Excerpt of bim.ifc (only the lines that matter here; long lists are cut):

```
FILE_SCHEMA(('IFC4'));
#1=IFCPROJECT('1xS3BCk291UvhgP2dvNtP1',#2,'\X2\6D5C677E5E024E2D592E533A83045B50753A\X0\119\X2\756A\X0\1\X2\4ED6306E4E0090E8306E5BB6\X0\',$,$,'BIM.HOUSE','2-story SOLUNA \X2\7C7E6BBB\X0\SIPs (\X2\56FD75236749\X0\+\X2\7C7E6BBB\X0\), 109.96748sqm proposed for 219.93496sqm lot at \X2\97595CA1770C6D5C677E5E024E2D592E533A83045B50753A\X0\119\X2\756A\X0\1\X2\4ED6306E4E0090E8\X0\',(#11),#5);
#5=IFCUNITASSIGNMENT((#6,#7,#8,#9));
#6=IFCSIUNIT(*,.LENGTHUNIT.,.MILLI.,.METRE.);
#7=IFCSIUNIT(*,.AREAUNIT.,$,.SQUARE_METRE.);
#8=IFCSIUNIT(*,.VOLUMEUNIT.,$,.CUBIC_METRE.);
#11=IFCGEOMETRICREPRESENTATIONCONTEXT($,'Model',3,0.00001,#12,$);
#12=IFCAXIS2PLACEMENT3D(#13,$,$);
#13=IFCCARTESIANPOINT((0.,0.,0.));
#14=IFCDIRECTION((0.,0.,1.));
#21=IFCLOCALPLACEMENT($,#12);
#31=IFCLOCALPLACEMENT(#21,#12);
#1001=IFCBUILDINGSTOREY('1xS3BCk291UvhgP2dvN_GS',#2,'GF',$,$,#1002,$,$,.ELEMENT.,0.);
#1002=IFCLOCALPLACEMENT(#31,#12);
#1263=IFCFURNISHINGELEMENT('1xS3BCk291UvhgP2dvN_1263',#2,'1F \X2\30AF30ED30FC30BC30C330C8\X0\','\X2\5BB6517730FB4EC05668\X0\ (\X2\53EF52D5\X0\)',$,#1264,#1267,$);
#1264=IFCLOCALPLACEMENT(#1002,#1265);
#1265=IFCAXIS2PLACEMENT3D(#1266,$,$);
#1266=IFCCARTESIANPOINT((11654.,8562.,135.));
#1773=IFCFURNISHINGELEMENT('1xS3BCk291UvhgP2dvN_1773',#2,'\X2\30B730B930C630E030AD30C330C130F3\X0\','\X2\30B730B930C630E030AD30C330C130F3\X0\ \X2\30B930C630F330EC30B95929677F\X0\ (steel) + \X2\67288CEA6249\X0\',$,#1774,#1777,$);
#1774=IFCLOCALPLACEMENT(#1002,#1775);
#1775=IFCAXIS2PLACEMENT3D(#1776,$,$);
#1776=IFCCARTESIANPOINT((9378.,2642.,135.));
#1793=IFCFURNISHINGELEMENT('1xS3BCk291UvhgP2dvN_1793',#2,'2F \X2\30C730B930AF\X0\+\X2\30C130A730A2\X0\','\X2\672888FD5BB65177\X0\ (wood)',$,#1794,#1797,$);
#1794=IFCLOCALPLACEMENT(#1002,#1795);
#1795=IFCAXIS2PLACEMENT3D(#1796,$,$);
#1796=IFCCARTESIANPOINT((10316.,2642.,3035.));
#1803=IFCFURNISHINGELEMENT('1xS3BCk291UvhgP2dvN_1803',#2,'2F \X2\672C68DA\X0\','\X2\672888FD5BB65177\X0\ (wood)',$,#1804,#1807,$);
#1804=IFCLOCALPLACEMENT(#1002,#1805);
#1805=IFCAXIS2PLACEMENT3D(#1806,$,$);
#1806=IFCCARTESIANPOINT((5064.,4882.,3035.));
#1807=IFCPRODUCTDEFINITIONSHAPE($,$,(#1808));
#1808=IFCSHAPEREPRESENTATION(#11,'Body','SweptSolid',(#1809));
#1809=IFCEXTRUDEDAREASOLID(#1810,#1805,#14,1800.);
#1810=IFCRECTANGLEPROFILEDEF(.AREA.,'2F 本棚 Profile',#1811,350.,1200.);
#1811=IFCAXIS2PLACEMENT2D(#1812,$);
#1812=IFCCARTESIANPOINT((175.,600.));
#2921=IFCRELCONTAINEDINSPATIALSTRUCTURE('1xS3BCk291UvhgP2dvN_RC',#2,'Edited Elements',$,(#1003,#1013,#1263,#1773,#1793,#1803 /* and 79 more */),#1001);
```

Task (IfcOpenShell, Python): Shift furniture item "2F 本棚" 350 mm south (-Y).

```python
import ifcopenshell
import ifcopenshell.api.geometry
import ifcopenshell.util.placement
import ifcopenshell.util.unit

model = ifcopenshell.open("bim.ifc")
unit_scale = ifcopenshell.util.unit.calculate_unit_scale(model)

item = model.by_id(1803)
matrix = ifcopenshell.util.placement.get_local_placement(item.ObjectPlacement)
matrix[1, 3] -= 0.35 / unit_scale
ifcopenshell.api.geometry.edit_object_placement(model, product=item, matrix=matrix, is_si=False)

print(ifcopenshell.util.placement.get_local_placement(item.ObjectPlacement).round(3) + 0.0)

model.write("bim_updated.ifc")
```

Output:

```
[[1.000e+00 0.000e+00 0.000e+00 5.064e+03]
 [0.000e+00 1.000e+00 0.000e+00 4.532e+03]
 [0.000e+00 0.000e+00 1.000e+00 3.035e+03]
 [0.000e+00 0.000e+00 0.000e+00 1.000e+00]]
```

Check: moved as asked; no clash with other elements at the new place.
